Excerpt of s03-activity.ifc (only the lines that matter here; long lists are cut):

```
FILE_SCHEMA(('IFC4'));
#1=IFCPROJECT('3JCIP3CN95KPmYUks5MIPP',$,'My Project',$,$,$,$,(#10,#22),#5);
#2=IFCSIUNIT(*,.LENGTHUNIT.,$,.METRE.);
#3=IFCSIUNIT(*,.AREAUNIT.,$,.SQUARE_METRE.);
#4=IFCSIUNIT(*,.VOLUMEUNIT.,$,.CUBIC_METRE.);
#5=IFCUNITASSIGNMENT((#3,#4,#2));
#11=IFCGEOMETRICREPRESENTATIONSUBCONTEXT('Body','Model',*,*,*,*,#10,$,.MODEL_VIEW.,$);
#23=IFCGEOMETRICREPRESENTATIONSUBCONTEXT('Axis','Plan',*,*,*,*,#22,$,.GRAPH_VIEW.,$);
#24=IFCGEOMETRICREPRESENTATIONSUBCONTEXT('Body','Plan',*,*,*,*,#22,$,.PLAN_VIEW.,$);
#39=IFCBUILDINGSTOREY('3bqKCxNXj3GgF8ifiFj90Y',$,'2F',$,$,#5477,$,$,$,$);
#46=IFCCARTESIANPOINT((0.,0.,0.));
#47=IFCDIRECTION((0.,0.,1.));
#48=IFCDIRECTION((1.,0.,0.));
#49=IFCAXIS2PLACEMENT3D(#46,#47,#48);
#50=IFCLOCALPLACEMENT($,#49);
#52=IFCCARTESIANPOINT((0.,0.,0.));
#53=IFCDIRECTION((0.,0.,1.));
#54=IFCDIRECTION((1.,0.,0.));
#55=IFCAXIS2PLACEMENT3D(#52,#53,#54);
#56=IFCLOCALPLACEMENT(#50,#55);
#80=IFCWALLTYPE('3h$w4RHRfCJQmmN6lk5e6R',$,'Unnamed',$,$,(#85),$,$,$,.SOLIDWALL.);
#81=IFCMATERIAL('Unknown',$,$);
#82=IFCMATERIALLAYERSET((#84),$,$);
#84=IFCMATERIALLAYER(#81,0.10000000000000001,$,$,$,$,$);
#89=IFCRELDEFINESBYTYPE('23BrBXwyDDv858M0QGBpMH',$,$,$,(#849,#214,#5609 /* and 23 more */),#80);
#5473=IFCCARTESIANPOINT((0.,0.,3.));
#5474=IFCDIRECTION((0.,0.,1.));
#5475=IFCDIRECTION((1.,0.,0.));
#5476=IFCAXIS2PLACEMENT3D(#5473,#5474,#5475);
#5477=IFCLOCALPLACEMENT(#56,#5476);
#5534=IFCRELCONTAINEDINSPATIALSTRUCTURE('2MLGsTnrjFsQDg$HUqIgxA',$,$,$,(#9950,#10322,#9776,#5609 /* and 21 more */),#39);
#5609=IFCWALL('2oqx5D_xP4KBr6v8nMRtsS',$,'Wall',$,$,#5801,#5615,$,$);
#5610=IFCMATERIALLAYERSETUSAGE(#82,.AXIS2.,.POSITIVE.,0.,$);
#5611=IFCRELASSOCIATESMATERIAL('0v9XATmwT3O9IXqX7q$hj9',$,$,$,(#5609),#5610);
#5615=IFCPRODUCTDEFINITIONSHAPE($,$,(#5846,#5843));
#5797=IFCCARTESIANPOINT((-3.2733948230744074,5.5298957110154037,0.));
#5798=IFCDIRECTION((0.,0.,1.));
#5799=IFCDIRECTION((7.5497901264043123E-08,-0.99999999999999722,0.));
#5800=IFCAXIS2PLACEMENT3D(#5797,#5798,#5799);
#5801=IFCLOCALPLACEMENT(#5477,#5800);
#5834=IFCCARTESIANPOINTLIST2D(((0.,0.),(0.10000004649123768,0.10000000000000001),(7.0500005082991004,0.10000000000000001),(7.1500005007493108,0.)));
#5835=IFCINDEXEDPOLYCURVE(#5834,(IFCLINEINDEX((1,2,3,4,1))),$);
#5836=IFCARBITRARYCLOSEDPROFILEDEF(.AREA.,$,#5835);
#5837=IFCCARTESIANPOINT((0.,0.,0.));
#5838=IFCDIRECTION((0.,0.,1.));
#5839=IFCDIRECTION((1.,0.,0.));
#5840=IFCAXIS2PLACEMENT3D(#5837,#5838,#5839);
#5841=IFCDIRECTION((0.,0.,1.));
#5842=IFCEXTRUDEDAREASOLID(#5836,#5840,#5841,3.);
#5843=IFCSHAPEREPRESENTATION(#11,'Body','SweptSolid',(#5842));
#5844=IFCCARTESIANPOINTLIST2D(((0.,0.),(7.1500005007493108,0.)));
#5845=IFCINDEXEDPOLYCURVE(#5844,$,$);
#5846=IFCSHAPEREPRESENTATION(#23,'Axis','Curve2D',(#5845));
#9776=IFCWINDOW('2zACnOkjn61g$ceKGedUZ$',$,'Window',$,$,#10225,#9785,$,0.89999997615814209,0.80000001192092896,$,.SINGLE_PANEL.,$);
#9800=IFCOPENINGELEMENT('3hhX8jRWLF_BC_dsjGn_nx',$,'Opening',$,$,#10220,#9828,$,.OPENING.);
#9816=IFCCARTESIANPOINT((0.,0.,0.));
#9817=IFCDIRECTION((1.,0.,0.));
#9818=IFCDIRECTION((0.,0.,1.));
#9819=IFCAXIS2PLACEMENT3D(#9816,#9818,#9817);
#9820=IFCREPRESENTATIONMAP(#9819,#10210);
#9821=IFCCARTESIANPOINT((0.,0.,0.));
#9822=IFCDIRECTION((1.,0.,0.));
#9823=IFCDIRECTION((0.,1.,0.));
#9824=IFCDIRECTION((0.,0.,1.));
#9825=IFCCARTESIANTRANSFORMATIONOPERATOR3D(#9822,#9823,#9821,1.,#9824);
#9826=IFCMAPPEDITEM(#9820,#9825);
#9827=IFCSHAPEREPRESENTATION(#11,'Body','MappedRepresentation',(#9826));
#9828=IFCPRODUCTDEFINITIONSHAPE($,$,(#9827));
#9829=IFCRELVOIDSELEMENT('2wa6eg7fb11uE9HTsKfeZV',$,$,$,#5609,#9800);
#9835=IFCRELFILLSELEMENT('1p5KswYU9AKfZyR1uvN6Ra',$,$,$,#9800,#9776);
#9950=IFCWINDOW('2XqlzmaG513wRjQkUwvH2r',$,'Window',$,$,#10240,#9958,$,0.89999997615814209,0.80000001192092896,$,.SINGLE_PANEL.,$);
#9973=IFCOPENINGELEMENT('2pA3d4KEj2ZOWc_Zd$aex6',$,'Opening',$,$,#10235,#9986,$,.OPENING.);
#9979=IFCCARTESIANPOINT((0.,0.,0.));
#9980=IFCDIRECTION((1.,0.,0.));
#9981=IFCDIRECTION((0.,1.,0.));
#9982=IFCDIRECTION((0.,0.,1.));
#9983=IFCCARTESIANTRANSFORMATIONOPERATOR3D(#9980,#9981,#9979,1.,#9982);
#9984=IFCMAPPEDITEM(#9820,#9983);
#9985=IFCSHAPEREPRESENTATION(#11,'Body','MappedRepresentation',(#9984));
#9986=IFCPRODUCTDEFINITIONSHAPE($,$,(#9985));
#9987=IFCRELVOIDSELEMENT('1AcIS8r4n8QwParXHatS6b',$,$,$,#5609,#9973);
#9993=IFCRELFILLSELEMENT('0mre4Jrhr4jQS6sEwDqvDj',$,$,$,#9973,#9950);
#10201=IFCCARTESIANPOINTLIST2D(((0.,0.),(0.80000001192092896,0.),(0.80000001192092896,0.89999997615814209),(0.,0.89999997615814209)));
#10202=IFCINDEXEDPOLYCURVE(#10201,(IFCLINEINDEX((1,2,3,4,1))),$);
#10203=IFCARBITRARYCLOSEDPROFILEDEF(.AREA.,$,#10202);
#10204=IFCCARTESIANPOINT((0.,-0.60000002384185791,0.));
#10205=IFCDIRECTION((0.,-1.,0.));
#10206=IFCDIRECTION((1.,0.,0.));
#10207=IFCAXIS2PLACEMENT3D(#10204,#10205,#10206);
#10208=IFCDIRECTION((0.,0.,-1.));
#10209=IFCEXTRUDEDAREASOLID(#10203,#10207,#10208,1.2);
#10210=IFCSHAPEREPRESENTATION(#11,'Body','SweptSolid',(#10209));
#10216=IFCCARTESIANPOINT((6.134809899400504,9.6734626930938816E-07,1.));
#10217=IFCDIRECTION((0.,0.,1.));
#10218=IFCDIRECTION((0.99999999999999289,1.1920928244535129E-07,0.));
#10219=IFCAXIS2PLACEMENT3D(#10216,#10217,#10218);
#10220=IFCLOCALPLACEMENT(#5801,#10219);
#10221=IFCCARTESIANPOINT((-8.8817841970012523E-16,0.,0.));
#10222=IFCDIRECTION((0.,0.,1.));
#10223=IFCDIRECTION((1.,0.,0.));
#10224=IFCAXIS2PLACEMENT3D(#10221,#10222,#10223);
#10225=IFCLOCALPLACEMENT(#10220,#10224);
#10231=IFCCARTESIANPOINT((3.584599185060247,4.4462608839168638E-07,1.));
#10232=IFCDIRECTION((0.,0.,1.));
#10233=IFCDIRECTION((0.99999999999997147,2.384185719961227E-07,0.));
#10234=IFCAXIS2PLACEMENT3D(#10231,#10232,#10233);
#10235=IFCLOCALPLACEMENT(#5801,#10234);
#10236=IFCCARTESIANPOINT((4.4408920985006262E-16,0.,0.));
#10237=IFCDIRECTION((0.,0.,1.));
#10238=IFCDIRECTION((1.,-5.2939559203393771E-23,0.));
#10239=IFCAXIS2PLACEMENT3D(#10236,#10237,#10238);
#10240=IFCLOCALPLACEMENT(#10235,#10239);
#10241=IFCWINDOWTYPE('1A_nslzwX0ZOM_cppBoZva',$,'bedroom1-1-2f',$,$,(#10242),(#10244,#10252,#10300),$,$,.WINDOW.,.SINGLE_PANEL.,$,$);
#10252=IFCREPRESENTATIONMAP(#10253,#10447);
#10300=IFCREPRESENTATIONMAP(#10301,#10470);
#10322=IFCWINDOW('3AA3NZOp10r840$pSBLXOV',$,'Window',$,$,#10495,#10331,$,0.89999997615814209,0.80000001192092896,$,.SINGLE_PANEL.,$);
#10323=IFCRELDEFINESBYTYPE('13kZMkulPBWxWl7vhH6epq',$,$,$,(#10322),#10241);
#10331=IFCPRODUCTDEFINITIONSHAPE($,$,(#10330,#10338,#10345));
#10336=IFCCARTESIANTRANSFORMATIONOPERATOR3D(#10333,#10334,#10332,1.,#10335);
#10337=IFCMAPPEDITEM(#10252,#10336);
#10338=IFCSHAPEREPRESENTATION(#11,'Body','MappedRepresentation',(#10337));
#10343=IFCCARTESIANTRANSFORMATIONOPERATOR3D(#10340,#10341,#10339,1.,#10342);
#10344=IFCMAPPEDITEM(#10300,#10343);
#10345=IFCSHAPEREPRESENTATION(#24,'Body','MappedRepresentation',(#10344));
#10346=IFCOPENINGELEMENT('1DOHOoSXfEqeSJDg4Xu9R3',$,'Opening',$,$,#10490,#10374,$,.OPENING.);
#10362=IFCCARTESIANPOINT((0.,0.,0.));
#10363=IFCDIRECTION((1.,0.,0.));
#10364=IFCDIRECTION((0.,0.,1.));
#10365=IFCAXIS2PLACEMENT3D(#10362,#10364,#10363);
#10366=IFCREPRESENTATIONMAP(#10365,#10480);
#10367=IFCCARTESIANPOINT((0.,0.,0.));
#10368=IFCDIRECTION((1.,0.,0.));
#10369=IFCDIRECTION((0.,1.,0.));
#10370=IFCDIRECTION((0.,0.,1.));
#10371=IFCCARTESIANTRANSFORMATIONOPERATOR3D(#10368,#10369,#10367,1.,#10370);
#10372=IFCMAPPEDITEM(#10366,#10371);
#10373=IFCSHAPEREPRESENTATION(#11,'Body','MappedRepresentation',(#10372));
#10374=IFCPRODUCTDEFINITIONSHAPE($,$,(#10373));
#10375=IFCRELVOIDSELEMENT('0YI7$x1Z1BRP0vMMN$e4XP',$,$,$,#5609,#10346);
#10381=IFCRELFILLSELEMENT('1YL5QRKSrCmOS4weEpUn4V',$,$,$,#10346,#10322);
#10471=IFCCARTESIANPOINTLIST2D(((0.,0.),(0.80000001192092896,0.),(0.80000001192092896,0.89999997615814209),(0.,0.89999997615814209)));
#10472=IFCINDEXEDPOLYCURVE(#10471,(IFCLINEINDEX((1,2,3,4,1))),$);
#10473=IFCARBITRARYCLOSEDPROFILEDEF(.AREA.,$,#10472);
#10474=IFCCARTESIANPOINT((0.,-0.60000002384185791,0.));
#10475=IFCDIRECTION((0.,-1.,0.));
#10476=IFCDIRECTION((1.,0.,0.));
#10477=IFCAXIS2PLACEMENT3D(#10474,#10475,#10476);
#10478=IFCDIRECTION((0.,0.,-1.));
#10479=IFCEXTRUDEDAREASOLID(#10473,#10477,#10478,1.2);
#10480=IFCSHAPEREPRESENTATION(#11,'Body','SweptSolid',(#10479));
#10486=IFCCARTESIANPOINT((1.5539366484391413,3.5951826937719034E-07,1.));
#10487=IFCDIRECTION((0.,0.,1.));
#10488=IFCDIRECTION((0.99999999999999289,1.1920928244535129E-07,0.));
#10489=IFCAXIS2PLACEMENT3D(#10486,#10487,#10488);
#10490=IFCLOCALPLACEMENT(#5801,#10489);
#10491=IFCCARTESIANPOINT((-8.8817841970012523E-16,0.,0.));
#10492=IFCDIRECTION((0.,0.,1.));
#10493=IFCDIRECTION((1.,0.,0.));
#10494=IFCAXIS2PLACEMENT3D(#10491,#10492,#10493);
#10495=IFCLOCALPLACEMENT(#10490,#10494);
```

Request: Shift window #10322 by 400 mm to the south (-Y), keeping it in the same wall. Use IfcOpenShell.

```python
import ifcopenshell
import ifcopenshell.api.geometry
import ifcopenshell.util.placement

model = ifcopenshell.open("s03-activity.ifc")

window = model.by_guid("3AA3NZOp10r840$pSBLXOV")
opening = window.FillsVoids[0].RelatingOpeningElement
wall = opening.VoidsElements[0].RelatingBuildingElement

wall_matrix = ifcopenshell.util.placement.get_local_placement(wall.ObjectPlacement)
shift = wall_matrix[:3, 0] * 0.4
before = ifcopenshell.util.placement.get_local_placement(window.ObjectPlacement)[:3, 3].copy()

# The window is placed relative to its opening, so it follows when the opening moves.
matrix = ifcopenshell.util.placement.get_local_placement(opening.ObjectPlacement)
matrix[:3, 3] += shift
ifcopenshell.api.geometry.edit_object_placement(
    model, product=opening, matrix=matrix, is_si=False, should_transform_children=True
)

after = ifcopenshell.util.placement.get_local_placement(window.ObjectPlacement)[:3, 3]
print("window moved by", (after - before).round(3) + 0.0)

model.write("s03-activity_rev.ifc")
```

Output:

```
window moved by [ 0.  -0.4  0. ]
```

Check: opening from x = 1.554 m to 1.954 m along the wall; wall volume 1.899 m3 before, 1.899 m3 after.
